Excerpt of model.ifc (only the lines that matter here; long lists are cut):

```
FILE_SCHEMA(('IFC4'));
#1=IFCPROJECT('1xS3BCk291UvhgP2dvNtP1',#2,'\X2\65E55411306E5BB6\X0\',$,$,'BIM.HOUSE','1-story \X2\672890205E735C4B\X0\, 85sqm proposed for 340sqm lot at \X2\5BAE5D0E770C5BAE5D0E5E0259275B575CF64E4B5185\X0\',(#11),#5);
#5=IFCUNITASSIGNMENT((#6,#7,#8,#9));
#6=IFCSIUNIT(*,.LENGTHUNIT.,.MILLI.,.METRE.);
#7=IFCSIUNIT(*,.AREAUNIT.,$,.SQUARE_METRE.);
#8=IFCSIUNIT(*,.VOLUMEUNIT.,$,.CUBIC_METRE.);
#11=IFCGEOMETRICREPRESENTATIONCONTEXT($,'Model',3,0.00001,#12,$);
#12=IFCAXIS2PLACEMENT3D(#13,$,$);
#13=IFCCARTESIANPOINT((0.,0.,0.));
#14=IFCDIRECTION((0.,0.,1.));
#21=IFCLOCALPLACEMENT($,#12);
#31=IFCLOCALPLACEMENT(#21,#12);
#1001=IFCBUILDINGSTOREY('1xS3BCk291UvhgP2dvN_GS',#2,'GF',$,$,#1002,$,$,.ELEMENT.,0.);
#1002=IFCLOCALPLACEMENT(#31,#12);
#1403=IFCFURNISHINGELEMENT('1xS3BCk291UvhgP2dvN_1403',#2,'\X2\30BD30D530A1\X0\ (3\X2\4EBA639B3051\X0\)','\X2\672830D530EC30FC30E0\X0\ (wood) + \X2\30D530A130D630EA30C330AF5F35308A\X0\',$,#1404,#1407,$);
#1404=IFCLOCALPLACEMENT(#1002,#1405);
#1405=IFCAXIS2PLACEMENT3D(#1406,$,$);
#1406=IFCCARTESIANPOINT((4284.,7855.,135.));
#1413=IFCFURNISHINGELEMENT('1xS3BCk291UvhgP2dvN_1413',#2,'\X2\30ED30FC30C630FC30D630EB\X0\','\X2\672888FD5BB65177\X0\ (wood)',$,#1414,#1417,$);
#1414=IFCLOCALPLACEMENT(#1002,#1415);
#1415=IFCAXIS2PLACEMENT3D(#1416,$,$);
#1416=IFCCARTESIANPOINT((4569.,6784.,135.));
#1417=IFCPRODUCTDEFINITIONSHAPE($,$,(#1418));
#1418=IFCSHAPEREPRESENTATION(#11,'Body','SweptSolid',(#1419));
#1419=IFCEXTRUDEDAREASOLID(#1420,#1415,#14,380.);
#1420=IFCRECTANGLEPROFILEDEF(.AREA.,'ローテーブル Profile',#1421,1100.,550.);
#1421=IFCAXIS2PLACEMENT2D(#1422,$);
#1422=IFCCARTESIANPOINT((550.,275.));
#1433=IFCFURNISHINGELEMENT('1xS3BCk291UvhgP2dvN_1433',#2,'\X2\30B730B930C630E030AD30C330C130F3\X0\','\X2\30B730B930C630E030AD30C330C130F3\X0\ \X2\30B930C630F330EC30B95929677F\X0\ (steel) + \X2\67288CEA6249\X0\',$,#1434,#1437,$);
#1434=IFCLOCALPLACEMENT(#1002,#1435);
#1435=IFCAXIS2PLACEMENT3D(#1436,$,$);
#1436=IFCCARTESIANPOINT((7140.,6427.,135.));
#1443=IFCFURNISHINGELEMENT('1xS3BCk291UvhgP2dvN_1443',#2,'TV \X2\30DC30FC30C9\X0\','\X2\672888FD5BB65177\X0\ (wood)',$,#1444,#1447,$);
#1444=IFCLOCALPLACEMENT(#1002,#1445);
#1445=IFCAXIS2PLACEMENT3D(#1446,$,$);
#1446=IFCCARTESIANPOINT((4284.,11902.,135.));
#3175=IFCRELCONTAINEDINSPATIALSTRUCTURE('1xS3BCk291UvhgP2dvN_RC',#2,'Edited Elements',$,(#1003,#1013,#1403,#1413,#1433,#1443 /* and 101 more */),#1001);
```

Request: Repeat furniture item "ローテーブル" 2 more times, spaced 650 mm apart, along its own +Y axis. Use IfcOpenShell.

```python
import ifcopenshell
import ifcopenshell.api.geometry
import ifcopenshell.api.root
import ifcopenshell.util.element
import ifcopenshell.util.placement
import ifcopenshell.util.unit

model = ifcopenshell.open("model.ifc")
unit_scale = ifcopenshell.util.unit.calculate_unit_scale(model)


def reuse_history(source, copy):
    """copy_class also copies each property set's owner history, people and application; keep the originals."""
    for rel in copy.IsDefinedBy:
        if rel.is_a("IfcRelDefinesByProperties") and (history := rel.RelatingPropertyDefinition.OwnerHistory):
            rel.RelatingPropertyDefinition.OwnerHistory = source.OwnerHistory
            ifcopenshell.util.element.remove_deep2(model, history)


source = model.by_guid("1xS3BCk291UvhgP2dvN_1413")
base = ifcopenshell.util.placement.get_local_placement(source.ObjectPlacement)
step = base[:3, 1] * 0.65 / unit_scale

for i in range(1, 3):
    copy = ifcopenshell.api.root.copy_class(model, product=source)
    copy.Representation = ifcopenshell.util.element.copy_deep(
        model, source.Representation, exclude=["IfcGeometricRepresentationContext", "IfcRepresentationMap"]
    )
    reuse_history(source, copy)
    matrix = base.copy()
    matrix[:3, 3] += i * step
    print("added at", matrix[:3, 3].round(3) + 0.0)
    ifcopenshell.api.geometry.edit_object_placement(model, product=copy, matrix=matrix, is_si=False)

model.write("model_rev.ifc")
```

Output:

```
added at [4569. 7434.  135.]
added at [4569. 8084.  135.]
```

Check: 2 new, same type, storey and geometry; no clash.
